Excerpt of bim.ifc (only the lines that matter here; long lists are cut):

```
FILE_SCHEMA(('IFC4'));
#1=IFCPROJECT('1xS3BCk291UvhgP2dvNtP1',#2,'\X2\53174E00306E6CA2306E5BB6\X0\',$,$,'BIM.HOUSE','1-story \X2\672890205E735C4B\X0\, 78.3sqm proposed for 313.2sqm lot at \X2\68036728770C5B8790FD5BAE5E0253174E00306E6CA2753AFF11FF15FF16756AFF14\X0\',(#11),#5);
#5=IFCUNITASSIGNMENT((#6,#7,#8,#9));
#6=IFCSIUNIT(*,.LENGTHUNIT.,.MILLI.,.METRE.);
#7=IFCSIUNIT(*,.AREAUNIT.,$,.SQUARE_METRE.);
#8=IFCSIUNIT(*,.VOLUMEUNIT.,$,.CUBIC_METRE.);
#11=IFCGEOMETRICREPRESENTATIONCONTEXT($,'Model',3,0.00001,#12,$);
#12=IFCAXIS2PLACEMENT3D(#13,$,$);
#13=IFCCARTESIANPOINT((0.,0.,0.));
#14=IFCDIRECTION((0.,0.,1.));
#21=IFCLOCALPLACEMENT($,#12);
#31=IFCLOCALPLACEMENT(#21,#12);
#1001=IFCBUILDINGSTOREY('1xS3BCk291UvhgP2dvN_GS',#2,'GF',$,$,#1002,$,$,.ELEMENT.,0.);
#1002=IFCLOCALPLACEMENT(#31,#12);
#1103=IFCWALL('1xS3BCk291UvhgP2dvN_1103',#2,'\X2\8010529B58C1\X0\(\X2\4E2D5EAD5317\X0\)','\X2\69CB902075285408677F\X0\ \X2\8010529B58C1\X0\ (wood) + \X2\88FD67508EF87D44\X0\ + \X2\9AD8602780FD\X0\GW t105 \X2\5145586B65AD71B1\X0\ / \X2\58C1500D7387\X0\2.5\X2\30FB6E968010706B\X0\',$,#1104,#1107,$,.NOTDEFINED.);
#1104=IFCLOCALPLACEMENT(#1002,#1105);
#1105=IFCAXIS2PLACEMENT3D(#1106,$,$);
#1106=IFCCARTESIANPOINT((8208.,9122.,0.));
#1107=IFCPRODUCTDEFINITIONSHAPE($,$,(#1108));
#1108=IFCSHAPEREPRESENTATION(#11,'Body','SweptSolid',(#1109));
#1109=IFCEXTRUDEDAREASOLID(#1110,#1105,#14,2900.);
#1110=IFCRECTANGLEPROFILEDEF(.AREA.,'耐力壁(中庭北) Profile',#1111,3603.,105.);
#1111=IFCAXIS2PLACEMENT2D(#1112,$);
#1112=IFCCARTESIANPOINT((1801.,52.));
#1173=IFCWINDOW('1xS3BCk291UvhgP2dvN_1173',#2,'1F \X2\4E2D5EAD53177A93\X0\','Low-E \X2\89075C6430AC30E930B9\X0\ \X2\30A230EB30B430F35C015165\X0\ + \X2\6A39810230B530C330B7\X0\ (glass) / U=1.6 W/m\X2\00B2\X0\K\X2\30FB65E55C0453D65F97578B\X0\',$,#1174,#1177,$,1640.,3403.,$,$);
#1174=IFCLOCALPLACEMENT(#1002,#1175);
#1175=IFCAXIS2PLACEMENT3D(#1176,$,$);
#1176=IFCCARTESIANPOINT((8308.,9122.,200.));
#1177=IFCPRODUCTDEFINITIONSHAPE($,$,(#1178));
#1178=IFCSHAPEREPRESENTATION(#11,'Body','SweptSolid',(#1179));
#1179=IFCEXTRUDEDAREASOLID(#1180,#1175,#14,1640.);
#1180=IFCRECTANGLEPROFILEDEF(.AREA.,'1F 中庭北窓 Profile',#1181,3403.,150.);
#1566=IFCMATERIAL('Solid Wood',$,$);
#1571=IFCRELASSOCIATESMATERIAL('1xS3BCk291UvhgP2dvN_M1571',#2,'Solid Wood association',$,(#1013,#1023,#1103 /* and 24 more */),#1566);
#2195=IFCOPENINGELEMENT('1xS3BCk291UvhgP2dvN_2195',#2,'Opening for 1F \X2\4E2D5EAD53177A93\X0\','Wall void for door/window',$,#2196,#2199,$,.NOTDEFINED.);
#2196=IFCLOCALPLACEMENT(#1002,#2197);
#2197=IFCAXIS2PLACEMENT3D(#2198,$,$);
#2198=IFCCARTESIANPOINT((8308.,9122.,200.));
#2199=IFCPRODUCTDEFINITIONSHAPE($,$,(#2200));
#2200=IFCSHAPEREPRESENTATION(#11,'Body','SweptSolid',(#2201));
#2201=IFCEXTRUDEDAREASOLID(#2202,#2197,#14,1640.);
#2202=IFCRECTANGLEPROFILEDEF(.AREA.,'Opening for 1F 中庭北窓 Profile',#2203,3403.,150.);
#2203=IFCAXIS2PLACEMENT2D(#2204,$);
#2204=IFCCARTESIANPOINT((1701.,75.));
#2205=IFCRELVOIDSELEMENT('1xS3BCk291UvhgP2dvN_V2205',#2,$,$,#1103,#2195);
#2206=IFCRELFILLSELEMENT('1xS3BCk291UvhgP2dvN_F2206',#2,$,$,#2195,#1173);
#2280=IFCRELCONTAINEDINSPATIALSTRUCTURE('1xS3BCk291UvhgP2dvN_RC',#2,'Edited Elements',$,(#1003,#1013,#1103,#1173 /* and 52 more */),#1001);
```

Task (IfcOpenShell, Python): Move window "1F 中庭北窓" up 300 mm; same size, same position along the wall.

```python
import numpy as np
import ifcopenshell
import ifcopenshell.api.geometry
import ifcopenshell.util.placement
import ifcopenshell.util.unit

model = ifcopenshell.open("bim.ifc")
unit_scale = ifcopenshell.util.unit.calculate_unit_scale(model)

window = model.by_guid("1xS3BCk291UvhgP2dvN_1173")
opening = window.FillsVoids[0].RelatingOpeningElement
dz = 300.0

shift = np.array([0.0, 0.0, dz])
# The window is not placed relative to its opening, so move both.
for product in (opening, window):
    matrix = ifcopenshell.util.placement.get_local_placement(product.ObjectPlacement)
    matrix[:3, 3] += shift
    ifcopenshell.api.geometry.edit_object_placement(model, product=product, matrix=matrix, is_si=False)

print(f"moved by {dz * unit_scale:+.3f} m")

model.write("bim_edited.ifc")
```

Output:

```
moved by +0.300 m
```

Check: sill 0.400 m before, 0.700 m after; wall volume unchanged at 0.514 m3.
